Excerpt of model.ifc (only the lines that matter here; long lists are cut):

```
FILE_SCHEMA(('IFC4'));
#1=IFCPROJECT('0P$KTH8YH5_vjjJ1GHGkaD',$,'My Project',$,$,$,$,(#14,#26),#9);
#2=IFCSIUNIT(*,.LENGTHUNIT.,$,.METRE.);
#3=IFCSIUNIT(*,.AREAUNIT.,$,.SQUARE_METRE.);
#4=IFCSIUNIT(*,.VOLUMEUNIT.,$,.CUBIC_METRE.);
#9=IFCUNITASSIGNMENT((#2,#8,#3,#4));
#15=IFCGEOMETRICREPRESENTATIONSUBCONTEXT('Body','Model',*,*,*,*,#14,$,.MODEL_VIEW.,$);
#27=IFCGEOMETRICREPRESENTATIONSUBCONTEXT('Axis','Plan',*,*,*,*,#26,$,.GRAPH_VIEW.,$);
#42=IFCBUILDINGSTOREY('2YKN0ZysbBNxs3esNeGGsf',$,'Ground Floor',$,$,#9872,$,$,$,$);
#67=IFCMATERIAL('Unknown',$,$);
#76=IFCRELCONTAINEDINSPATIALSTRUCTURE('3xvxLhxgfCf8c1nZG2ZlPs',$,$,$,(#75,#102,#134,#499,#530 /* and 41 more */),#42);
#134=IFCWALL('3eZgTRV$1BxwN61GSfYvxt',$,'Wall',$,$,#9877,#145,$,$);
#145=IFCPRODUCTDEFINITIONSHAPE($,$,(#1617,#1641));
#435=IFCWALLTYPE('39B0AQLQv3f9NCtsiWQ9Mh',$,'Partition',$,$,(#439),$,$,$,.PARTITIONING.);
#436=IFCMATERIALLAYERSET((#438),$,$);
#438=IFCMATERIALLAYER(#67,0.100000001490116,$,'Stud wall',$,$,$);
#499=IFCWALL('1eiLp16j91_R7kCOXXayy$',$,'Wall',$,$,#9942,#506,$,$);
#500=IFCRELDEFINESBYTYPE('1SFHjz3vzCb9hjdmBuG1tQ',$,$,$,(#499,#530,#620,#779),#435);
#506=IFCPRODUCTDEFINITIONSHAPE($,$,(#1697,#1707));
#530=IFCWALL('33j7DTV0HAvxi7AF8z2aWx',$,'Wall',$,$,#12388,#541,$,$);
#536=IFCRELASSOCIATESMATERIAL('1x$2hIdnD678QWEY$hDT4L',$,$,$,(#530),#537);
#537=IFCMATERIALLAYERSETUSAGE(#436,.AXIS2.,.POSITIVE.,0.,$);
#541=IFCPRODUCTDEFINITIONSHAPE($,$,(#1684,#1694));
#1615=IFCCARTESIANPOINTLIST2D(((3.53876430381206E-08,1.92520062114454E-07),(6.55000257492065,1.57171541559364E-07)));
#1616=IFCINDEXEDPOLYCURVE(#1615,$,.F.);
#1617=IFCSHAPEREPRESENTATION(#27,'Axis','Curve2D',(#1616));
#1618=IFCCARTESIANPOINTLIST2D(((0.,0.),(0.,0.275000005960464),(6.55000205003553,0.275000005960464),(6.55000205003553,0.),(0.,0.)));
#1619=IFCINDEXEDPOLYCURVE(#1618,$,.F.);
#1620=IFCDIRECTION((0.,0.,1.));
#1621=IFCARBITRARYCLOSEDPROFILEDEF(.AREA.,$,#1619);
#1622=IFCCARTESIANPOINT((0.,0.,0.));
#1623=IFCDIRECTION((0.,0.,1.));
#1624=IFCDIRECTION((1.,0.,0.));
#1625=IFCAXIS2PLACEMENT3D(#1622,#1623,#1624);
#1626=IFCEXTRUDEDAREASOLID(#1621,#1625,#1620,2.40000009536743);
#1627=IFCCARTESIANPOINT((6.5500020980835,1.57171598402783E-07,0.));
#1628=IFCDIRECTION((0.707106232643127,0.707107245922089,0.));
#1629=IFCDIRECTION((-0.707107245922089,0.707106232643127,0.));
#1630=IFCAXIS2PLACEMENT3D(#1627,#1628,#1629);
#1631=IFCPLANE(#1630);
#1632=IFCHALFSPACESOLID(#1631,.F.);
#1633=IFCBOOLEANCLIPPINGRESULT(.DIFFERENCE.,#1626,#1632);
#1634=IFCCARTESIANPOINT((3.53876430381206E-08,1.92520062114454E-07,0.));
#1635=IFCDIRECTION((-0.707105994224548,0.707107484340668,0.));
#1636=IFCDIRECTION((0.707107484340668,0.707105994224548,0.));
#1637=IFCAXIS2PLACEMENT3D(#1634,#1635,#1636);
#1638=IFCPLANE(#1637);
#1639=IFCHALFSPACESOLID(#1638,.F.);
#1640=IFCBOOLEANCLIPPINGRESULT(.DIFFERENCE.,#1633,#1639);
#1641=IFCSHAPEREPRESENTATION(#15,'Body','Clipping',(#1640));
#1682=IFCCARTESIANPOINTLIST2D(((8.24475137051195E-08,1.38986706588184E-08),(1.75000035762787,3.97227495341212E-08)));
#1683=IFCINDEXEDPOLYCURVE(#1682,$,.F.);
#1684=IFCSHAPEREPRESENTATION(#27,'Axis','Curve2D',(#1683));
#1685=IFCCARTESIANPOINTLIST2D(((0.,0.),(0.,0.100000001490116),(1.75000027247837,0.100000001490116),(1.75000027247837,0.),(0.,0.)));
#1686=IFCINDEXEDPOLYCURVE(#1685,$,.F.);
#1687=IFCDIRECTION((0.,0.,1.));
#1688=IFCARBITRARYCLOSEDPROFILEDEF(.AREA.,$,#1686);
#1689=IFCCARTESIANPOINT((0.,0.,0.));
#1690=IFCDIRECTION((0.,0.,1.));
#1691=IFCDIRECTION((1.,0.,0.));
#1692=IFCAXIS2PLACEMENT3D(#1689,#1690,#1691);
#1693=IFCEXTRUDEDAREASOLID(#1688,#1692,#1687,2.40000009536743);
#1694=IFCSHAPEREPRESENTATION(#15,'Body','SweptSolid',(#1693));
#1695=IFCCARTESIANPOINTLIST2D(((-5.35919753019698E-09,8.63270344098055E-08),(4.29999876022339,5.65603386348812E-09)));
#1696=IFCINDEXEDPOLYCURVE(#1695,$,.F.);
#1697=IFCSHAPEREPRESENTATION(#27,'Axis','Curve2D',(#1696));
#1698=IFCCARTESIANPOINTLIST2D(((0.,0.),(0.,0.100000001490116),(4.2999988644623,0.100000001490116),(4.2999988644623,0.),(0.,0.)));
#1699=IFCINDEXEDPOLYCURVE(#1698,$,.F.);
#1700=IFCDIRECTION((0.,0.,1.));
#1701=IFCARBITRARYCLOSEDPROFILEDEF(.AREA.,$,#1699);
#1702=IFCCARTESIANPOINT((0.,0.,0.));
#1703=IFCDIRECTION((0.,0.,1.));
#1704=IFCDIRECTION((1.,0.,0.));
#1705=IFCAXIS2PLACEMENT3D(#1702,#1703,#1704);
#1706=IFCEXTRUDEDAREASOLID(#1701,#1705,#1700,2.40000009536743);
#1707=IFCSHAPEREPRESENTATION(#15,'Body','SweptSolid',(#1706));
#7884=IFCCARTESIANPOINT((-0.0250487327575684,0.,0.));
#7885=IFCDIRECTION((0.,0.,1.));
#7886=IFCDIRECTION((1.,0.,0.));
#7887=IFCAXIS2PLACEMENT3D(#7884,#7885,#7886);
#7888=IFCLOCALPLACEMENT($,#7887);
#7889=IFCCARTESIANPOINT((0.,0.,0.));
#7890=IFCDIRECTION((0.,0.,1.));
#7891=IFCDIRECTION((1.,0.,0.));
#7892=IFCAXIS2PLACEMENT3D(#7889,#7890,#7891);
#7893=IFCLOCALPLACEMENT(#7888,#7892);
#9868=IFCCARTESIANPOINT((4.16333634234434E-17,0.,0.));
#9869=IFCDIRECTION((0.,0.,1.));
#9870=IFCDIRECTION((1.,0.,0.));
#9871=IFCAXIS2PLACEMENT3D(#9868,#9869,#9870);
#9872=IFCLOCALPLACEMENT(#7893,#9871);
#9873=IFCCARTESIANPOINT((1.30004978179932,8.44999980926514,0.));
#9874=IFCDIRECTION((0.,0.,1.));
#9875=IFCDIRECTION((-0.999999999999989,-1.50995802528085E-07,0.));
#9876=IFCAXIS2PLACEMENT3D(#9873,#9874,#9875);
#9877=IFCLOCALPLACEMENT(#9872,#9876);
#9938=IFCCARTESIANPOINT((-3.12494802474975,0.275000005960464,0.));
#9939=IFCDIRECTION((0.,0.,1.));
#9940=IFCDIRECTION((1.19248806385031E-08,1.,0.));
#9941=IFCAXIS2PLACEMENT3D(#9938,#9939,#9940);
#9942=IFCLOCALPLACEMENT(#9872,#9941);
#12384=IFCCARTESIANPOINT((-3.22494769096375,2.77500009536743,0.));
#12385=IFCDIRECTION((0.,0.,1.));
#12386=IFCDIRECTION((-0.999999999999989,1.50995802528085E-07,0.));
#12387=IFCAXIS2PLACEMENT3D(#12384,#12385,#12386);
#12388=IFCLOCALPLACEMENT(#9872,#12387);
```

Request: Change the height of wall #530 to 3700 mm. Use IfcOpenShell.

```python
import ifcopenshell
import ifcopenshell.geom
import ifcopenshell.util.representation
import ifcopenshell.util.shape
import ifcopenshell.util.unit

model = ifcopenshell.open("model.ifc")
unit_scale = ifcopenshell.util.unit.calculate_unit_scale(model)
settings = ifcopenshell.geom.settings()


def volume(element):
    """Net volume in cubic metres, openings subtracted."""
    shape = ifcopenshell.geom.create_shape(settings, element)
    return ifcopenshell.util.shape.get_volume(shape.geometry)


wall = model.by_guid("33j7DTV0HAvxi7AF8z2aWx")
before = volume(wall)

body = ifcopenshell.util.representation.get_representation(wall, "Model", "Body")
solid = body.Items[0]
old_height = solid.Depth
solid.Depth = 3.7 / unit_scale
after = volume(wall)

print(f"height {old_height:g} -> {solid.Depth:g}, volume {before:.3f} -> {after:.3f} m3")

model.write("model_edited.ifc")
```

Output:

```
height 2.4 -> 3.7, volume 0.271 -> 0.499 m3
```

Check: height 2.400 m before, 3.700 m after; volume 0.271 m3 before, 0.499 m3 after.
